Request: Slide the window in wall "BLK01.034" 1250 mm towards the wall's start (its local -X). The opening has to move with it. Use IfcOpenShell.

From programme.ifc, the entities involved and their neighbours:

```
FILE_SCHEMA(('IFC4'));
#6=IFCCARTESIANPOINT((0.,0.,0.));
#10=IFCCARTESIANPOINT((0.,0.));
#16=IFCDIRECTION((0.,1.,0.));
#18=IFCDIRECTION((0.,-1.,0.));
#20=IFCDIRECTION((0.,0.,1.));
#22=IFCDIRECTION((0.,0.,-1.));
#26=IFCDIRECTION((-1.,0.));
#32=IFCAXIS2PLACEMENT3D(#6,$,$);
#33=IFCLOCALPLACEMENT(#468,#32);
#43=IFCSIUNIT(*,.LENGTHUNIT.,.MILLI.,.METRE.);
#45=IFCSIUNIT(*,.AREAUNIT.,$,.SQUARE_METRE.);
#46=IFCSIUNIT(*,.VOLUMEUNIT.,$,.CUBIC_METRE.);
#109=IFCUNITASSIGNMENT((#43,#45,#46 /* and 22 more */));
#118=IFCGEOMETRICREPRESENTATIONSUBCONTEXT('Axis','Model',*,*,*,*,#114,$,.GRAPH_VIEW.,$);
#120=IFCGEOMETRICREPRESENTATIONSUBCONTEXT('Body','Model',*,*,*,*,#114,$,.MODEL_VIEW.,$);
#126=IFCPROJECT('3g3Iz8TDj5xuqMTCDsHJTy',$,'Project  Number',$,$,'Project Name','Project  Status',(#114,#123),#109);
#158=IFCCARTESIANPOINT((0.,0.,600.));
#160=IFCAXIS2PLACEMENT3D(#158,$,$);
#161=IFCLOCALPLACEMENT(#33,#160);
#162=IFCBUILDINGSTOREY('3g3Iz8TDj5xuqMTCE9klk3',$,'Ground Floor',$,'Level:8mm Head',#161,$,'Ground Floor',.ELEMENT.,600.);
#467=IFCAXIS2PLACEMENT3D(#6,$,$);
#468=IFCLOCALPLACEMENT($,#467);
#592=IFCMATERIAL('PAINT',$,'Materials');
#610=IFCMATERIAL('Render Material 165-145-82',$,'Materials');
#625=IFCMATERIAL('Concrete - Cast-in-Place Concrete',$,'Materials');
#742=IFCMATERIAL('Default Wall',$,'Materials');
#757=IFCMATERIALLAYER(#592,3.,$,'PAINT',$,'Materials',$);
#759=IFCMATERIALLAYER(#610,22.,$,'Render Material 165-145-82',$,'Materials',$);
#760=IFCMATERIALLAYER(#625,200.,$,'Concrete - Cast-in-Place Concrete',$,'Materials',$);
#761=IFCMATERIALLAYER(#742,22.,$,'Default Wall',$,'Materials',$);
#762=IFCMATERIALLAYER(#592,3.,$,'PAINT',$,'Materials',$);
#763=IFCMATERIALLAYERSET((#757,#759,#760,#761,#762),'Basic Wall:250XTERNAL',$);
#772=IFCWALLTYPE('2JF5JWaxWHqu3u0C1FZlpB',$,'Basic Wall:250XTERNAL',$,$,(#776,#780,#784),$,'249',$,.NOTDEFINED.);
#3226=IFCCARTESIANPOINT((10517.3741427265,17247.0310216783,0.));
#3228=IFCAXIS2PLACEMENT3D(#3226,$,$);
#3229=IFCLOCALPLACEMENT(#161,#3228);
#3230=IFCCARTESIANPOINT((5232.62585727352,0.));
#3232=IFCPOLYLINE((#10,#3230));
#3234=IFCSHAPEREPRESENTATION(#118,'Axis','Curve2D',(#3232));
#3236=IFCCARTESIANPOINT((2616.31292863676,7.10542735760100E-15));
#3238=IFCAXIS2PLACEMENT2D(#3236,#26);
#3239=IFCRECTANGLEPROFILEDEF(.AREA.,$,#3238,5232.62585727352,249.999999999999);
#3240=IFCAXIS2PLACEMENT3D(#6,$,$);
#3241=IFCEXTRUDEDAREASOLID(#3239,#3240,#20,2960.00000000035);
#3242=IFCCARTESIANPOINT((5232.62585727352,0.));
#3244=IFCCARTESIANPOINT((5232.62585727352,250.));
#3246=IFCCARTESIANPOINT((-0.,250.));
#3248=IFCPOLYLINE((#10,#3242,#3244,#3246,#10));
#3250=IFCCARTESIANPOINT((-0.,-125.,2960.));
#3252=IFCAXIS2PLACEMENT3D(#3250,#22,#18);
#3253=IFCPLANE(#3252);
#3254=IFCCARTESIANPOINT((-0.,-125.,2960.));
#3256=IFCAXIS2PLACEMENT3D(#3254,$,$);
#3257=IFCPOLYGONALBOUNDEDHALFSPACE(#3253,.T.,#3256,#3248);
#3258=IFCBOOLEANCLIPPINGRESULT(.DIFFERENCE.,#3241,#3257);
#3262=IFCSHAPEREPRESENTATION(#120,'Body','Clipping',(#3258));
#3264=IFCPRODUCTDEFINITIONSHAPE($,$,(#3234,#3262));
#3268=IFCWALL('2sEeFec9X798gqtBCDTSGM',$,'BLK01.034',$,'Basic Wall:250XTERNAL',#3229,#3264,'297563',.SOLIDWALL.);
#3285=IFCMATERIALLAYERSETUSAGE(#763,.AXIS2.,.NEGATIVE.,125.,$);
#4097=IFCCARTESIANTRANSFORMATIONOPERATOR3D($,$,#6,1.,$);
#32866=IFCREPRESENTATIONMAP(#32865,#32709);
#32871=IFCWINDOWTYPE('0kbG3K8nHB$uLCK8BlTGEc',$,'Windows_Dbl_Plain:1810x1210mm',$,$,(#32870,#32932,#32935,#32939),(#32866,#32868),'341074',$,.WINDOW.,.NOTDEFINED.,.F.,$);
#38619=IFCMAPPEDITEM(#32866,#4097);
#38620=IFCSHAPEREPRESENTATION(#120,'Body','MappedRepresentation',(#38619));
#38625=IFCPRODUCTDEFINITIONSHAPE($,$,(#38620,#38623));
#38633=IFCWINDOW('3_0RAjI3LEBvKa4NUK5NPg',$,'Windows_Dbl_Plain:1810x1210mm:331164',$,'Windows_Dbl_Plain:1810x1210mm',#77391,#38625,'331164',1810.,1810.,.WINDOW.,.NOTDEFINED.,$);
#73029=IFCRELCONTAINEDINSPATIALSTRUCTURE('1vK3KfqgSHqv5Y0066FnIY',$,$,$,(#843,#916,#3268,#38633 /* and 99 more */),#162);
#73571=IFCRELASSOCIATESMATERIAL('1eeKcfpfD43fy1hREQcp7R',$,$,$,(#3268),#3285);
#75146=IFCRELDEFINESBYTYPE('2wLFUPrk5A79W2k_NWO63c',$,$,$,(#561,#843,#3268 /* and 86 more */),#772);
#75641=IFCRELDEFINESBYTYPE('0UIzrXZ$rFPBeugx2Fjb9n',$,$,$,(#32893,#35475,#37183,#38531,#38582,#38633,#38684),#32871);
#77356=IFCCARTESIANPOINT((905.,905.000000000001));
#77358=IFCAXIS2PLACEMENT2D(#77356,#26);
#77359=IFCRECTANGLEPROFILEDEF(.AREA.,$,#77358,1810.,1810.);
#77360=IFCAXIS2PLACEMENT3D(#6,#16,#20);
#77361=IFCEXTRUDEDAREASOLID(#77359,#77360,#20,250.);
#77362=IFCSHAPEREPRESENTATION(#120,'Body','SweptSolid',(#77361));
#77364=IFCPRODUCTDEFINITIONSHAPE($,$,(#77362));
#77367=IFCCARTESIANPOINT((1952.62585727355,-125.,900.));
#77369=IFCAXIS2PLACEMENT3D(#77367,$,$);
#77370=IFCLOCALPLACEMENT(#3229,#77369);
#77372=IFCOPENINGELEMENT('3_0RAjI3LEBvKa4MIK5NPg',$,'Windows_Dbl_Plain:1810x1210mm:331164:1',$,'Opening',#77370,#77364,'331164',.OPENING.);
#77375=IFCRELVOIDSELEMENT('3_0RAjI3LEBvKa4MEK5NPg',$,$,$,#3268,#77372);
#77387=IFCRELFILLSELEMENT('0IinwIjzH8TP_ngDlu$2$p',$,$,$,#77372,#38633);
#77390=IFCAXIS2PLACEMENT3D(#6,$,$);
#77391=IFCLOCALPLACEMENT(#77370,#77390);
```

```python
import ifcopenshell
import ifcopenshell.api.geometry
import ifcopenshell.util.placement
import ifcopenshell.util.unit

model = ifcopenshell.open("programme.ifc")
unit_scale = ifcopenshell.util.unit.calculate_unit_scale(model)

window = model.by_guid("3_0RAjI3LEBvKa4NUK5NPg")
opening = window.FillsVoids[0].RelatingOpeningElement
wall = opening.VoidsElements[0].RelatingBuildingElement

wall_matrix = ifcopenshell.util.placement.get_local_placement(wall.ObjectPlacement)
shift = wall_matrix[:3, 0] * -1.25 / unit_scale
before = ifcopenshell.util.placement.get_local_placement(window.ObjectPlacement)[:3, 3].copy()

# The window is placed relative to its opening, so it follows when the opening moves.
matrix = ifcopenshell.util.placement.get_local_placement(opening.ObjectPlacement)
matrix[:3, 3] += shift
ifcopenshell.api.geometry.edit_object_placement(
    model, product=opening, matrix=matrix, is_si=False, should_transform_children=True
)

after = ifcopenshell.util.placement.get_local_placement(window.ObjectPlacement)[:3, 3]
print("window moved by", (after - before).round(3) + 0.0)

model.write("programme_v2.ifc")
```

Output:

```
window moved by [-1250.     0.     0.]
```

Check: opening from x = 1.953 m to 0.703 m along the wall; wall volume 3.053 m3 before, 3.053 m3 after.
